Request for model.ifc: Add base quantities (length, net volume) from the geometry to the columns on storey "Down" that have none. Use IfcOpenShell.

First a look at what the model holds.

```python
import ifcopenshell
import ifcopenshell.util.element
import ifcopenshell.util.unit

model = ifcopenshell.open("model.ifc")
print(model.schema)
for unit_type in ("LENGTHUNIT", "AREAUNIT", "VOLUMEUNIT"):
    print(unit_type, ifcopenshell.util.unit.calculate_unit_scale(model, unit_type))
storey = next(s for s in model.by_type("IfcBuildingStorey") if s.Name == "Down")
columns = [e for e in ifcopenshell.util.element.get_decomposition(storey) if e.is_a("IfcColumn")]
for e in sorted(columns, key=lambda e: e.id()):
    print(e.id(), e.is_a(), e.Name, list(ifcopenshell.util.element.get_psets(e, qtos_only=True)), sep=" | ")
```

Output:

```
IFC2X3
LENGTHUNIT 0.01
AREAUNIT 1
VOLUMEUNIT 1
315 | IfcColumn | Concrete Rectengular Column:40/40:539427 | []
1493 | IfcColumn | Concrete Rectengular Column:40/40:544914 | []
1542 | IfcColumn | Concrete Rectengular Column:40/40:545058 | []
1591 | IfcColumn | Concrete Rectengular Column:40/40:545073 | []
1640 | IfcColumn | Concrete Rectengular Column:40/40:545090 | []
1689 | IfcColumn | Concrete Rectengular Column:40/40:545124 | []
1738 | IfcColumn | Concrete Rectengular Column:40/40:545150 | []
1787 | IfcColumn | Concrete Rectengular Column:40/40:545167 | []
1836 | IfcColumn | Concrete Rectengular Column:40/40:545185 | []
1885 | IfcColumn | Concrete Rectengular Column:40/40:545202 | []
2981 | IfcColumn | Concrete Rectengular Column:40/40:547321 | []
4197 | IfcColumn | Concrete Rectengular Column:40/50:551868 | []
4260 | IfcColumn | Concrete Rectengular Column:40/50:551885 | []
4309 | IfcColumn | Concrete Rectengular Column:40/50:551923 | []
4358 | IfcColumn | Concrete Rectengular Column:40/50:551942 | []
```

```python
import ifcopenshell
import ifcopenshell.api.pset
import ifcopenshell.geom
import ifcopenshell.util.element
import ifcopenshell.util.shape
import ifcopenshell.util.unit

model = ifcopenshell.open("model.ifc")
unit_scale = ifcopenshell.util.unit.calculate_unit_scale(model)
volume_scale = ifcopenshell.util.unit.calculate_unit_scale(model, "VOLUMEUNIT")
settings = ifcopenshell.geom.settings()

storey = next(s for s in model.by_type("IfcBuildingStorey") if s.Name == "Down")
columns = [e for e in ifcopenshell.util.element.get_decomposition(storey) if e.is_a("IfcColumn")]

for e in sorted(columns, key=lambda e: e.id()):
    if ifcopenshell.util.element.get_psets(e, qtos_only=True, should_inherit=False):
        continue
    # Geometry comes back in metres, in the element's own axes.
    shape = ifcopenshell.geom.create_shape(settings, e)
    values = {
        "Length": ifcopenshell.util.shape.get_z(shape.geometry) / unit_scale,
        "NetVolume": ifcopenshell.util.shape.get_volume(shape.geometry) / volume_scale,
    }
    qto = ifcopenshell.api.pset.add_qto(model, product=e, name="BaseQuantities")
    ifcopenshell.api.pset.edit_qto(model, qto=qto, properties=values)
    print(e.id(), {k: round(v, 3) for k, v in values.items()})

model.write("model_v2.ifc")
```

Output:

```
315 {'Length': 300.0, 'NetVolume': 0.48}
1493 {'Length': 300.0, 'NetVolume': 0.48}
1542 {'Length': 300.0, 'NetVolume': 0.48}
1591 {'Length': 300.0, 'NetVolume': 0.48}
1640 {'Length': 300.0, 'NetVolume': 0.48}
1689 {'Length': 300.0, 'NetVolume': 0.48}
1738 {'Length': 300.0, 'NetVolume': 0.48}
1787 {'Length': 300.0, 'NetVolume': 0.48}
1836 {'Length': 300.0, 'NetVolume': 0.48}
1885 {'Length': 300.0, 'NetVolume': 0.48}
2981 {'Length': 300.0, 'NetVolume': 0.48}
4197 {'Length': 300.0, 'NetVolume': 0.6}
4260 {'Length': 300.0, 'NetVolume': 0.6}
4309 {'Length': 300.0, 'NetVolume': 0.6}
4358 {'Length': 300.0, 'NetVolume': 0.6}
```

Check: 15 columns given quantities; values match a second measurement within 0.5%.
